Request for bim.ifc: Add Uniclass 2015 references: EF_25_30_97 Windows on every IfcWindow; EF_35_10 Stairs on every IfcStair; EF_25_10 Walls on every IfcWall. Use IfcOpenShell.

First a look at what the model holds.

```python
import ifcopenshell

model = ifcopenshell.open("bim.ifc")
print(model.schema)
print("classifications:", [c.Name for c in model.by_type("IfcClassification")])
for ifc_class in ("IfcDoor", "IfcRoof", "IfcStair", "IfcWall", "IfcWindow"):
    print(ifc_class, len(model.by_type(ifc_class)))
```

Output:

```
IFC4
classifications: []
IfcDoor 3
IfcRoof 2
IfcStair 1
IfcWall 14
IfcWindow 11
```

```python
import ifcopenshell
import ifcopenshell.api.classification

model = ifcopenshell.open("bim.ifc")

system = ifcopenshell.api.classification.add_classification(model, classification="Uniclass 2015")

codes = {
    "IfcWindow": ("EF_25_30_97", "Windows"),
    "IfcStair": ("EF_35_10", "Stairs"),
    "IfcWall": ("EF_25_10", "Walls"),
}
for ifc_class, (code, name) in codes.items():
    products = model.by_type(ifc_class)
    ifcopenshell.api.classification.add_reference(
        model, products=products, classification=system, identification=code, name=name
    )
    print(code, len(products))

model.write("bim_v2.ifc")
```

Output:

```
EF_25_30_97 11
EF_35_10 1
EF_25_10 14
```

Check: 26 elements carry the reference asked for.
